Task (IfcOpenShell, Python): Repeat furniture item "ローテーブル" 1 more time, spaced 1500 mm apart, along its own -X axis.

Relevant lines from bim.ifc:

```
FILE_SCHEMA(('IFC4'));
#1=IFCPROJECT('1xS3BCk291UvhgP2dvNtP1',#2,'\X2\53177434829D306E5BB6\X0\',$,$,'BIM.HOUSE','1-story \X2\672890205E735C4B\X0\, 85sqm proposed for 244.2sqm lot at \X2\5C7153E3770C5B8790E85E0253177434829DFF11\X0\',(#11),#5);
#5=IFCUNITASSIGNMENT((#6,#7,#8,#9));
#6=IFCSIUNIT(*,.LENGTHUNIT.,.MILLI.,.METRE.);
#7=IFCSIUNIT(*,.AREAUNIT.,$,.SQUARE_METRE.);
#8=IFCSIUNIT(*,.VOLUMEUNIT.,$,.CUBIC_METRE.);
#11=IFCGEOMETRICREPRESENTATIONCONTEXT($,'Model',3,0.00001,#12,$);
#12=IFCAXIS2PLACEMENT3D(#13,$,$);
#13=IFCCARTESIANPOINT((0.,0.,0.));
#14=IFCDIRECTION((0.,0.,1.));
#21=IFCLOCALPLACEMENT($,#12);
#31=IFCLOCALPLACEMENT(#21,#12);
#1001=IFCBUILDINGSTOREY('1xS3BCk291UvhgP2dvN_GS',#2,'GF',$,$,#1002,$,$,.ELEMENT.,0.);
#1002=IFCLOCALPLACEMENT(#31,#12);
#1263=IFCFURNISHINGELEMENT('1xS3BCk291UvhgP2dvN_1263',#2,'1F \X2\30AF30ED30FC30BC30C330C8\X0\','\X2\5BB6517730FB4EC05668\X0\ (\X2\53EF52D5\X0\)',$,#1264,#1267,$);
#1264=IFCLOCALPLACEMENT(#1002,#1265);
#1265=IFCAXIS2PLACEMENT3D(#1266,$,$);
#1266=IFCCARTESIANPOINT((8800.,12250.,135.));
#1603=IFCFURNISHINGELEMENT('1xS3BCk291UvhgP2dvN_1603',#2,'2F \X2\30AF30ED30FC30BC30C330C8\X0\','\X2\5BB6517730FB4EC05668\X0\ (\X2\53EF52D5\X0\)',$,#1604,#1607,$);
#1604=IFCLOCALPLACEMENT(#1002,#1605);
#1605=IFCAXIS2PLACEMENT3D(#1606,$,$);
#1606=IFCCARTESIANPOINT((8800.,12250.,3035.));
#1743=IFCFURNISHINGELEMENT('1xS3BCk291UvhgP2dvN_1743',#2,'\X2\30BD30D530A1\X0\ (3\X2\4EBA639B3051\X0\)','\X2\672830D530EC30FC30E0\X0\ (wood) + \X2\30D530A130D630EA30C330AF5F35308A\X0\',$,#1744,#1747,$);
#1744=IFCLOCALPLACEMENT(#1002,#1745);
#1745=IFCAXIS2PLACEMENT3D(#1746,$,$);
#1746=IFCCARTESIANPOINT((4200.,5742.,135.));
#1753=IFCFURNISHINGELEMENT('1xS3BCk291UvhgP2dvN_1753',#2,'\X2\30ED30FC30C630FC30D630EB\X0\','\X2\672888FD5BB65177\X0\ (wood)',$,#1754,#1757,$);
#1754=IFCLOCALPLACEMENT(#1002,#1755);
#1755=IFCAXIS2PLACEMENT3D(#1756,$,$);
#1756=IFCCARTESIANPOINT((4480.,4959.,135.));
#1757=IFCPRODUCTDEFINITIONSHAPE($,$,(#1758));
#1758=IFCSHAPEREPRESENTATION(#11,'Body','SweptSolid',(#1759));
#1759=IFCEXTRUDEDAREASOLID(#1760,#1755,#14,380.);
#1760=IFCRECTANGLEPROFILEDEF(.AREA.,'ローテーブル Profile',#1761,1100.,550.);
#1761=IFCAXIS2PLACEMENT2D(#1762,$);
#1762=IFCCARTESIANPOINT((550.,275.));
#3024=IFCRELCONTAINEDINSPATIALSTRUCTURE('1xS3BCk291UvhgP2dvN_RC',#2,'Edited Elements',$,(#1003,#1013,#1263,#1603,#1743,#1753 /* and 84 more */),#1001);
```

```python
import ifcopenshell
import ifcopenshell.api.geometry
import ifcopenshell.api.root
import ifcopenshell.util.element
import ifcopenshell.util.placement
import ifcopenshell.util.unit

model = ifcopenshell.open("bim.ifc")
unit_scale = ifcopenshell.util.unit.calculate_unit_scale(model)


def reuse_history(source, copy):
    """copy_class also copies each property set's owner history, people and application; keep the originals."""
    for rel in copy.IsDefinedBy:
        if rel.is_a("IfcRelDefinesByProperties") and (history := rel.RelatingPropertyDefinition.OwnerHistory):
            rel.RelatingPropertyDefinition.OwnerHistory = source.OwnerHistory
            ifcopenshell.util.element.remove_deep2(model, history)


source = model.by_guid("1xS3BCk291UvhgP2dvN_1753")
base = ifcopenshell.util.placement.get_local_placement(source.ObjectPlacement)
step = -base[:3, 0] * 1.5 / unit_scale

for i in range(1, 2):
    copy = ifcopenshell.api.root.copy_class(model, product=source)
    copy.Representation = ifcopenshell.util.element.copy_deep(
        model, source.Representation, exclude=["IfcGeometricRepresentationContext", "IfcRepresentationMap"]
    )
    reuse_history(source, copy)
    matrix = base.copy()
    matrix[:3, 3] += i * step
    print("added at", matrix[:3, 3].round(3) + 0.0)
    ifcopenshell.api.geometry.edit_object_placement(model, product=copy, matrix=matrix, is_si=False)

model.write("bim_rev.ifc")
```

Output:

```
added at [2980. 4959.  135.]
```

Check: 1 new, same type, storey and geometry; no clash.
